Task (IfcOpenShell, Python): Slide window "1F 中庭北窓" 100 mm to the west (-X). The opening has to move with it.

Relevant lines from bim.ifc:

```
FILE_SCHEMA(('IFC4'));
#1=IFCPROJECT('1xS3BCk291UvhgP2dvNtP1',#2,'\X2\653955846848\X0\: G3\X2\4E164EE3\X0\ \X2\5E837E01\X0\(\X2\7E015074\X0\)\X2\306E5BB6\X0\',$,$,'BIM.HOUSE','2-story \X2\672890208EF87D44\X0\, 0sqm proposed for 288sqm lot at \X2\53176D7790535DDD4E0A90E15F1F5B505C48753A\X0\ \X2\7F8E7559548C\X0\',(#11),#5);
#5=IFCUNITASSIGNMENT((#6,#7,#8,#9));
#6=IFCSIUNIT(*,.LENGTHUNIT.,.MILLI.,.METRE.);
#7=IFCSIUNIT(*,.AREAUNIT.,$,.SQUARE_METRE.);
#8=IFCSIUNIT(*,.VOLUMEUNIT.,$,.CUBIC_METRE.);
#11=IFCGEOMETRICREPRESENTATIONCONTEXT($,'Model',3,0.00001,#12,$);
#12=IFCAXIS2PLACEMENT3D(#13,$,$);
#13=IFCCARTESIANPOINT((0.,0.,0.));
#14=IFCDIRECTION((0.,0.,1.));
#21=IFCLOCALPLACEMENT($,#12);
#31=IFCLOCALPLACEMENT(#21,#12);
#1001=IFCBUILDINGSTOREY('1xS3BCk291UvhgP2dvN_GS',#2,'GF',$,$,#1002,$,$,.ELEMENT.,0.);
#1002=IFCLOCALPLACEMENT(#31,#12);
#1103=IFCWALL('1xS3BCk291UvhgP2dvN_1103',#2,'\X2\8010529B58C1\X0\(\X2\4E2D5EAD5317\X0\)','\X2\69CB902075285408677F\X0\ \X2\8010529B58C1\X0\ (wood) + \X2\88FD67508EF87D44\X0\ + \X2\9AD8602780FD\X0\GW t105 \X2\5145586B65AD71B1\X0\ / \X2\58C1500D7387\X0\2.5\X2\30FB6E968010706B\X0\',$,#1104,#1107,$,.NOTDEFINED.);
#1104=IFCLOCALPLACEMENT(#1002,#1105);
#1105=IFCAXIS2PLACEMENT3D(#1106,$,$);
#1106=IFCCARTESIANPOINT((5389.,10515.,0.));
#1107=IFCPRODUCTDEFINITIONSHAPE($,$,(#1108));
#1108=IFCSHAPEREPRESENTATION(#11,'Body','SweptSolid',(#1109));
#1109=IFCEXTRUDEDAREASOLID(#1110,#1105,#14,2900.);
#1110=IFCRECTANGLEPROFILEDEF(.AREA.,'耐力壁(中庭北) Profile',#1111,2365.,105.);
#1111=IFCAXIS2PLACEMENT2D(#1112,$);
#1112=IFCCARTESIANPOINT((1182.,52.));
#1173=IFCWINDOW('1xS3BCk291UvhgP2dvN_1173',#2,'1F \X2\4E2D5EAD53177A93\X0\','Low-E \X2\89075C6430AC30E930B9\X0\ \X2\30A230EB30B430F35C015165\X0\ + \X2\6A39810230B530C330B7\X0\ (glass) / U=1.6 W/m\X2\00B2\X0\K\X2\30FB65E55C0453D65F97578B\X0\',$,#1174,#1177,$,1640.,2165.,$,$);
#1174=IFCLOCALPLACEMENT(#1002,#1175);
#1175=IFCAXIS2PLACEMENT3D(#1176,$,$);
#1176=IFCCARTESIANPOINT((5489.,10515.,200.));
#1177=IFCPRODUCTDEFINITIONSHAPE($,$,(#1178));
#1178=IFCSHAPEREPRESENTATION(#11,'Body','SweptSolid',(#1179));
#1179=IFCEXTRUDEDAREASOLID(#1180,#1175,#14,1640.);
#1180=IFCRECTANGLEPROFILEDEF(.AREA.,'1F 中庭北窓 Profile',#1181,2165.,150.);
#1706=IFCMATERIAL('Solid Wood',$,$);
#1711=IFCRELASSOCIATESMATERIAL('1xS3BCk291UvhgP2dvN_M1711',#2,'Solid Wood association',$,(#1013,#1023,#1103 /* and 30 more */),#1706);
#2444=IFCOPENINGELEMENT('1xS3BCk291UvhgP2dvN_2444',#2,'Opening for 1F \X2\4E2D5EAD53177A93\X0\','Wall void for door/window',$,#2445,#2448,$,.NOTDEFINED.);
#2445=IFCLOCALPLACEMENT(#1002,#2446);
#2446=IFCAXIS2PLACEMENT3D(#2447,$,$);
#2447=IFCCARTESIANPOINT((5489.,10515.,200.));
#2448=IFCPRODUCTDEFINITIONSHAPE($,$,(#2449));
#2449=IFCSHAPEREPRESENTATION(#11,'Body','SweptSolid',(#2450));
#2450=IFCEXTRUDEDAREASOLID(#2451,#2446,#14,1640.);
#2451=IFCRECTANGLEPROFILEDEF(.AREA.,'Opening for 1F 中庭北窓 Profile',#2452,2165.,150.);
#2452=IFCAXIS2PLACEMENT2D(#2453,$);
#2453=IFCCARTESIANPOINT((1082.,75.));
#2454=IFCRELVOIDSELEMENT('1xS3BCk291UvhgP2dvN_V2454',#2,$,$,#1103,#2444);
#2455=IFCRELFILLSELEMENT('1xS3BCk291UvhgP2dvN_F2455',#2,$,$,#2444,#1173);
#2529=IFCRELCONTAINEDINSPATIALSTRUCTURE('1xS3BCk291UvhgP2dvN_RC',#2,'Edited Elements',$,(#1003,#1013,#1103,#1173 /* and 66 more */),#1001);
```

```python
import ifcopenshell
import ifcopenshell.api.geometry
import ifcopenshell.util.placement

model = ifcopenshell.open("bim.ifc")

window = model.by_guid("1xS3BCk291UvhgP2dvN_1173")
opening = window.FillsVoids[0].RelatingOpeningElement
wall = opening.VoidsElements[0].RelatingBuildingElement

wall_matrix = ifcopenshell.util.placement.get_local_placement(wall.ObjectPlacement)
shift = wall_matrix[:3, 0] * -100.0
before = ifcopenshell.util.placement.get_local_placement(window.ObjectPlacement)[:3, 3].copy()

# The window is not placed relative to its opening, so move both.
for product in (opening, window):
    matrix = ifcopenshell.util.placement.get_local_placement(product.ObjectPlacement)
    matrix[:3, 3] += shift
    ifcopenshell.api.geometry.edit_object_placement(model, product=product, matrix=matrix, is_si=False)

after = ifcopenshell.util.placement.get_local_placement(window.ObjectPlacement)[:3, 3]
print("window moved by", (after - before).round(3) + 0.0)

model.write("bim-out.ifc")
```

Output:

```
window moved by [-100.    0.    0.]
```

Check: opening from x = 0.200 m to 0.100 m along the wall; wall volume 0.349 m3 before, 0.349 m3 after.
